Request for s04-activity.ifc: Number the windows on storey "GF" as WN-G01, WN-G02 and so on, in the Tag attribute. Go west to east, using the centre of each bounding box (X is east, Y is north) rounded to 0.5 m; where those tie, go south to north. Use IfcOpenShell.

First a look at what the model holds.

```python
import ifcopenshell
import ifcopenshell.util.element
import ifcopenshell.util.placement

model = ifcopenshell.open("s04-activity.ifc")
print(model.schema)
storey = next(s for s in model.by_type("IfcBuildingStorey") if s.Name == "GF")
windows = [e for e in ifcopenshell.util.element.get_decomposition(storey) if e.is_a("IfcWindow")]
for e in sorted(windows, key=lambda e: e.id()):
    origin = ifcopenshell.util.placement.get_local_placement(e.ObjectPlacement)[:3, 3]
    print(e.id(), e.Tag, e.Name, origin.round(2) + 0.0, sep=" | ")
```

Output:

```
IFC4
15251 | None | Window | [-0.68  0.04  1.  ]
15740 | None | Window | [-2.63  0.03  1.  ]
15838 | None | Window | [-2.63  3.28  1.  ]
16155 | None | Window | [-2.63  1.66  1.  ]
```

```python
import ifcopenshell
import ifcopenshell.geom
import ifcopenshell.util.element
import ifcopenshell.util.shape

model = ifcopenshell.open("s04-activity.ifc")
settings = ifcopenshell.geom.settings()
settings.set("use-world-coords", True)


def centre(element):
    shape = ifcopenshell.geom.create_shape(settings, element)
    return ifcopenshell.util.shape.get_bbox_centroid(shape.geometry)


storey = next(s for s in model.by_type("IfcBuildingStorey") if s.Name == "GF")
windows = [e for e in ifcopenshell.util.element.get_decomposition(storey) if e.is_a("IfcWindow")]

# Insertion points can sit at a corner or the storey origin, so sort by the geometry (in metres).
centres = {e: centre(e) for e in windows}
windows.sort(key=lambda e: (round(centres[e][0] / 0.5), centres[e][1]))

for i, e in enumerate(windows, start=1):
    number = f"WN-G{i:02d}"
    e.Tag = number
    print(e.id(), number)

model.write("s04-activity-out.ifc")
```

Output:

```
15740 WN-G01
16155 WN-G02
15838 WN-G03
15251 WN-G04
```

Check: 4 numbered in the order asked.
